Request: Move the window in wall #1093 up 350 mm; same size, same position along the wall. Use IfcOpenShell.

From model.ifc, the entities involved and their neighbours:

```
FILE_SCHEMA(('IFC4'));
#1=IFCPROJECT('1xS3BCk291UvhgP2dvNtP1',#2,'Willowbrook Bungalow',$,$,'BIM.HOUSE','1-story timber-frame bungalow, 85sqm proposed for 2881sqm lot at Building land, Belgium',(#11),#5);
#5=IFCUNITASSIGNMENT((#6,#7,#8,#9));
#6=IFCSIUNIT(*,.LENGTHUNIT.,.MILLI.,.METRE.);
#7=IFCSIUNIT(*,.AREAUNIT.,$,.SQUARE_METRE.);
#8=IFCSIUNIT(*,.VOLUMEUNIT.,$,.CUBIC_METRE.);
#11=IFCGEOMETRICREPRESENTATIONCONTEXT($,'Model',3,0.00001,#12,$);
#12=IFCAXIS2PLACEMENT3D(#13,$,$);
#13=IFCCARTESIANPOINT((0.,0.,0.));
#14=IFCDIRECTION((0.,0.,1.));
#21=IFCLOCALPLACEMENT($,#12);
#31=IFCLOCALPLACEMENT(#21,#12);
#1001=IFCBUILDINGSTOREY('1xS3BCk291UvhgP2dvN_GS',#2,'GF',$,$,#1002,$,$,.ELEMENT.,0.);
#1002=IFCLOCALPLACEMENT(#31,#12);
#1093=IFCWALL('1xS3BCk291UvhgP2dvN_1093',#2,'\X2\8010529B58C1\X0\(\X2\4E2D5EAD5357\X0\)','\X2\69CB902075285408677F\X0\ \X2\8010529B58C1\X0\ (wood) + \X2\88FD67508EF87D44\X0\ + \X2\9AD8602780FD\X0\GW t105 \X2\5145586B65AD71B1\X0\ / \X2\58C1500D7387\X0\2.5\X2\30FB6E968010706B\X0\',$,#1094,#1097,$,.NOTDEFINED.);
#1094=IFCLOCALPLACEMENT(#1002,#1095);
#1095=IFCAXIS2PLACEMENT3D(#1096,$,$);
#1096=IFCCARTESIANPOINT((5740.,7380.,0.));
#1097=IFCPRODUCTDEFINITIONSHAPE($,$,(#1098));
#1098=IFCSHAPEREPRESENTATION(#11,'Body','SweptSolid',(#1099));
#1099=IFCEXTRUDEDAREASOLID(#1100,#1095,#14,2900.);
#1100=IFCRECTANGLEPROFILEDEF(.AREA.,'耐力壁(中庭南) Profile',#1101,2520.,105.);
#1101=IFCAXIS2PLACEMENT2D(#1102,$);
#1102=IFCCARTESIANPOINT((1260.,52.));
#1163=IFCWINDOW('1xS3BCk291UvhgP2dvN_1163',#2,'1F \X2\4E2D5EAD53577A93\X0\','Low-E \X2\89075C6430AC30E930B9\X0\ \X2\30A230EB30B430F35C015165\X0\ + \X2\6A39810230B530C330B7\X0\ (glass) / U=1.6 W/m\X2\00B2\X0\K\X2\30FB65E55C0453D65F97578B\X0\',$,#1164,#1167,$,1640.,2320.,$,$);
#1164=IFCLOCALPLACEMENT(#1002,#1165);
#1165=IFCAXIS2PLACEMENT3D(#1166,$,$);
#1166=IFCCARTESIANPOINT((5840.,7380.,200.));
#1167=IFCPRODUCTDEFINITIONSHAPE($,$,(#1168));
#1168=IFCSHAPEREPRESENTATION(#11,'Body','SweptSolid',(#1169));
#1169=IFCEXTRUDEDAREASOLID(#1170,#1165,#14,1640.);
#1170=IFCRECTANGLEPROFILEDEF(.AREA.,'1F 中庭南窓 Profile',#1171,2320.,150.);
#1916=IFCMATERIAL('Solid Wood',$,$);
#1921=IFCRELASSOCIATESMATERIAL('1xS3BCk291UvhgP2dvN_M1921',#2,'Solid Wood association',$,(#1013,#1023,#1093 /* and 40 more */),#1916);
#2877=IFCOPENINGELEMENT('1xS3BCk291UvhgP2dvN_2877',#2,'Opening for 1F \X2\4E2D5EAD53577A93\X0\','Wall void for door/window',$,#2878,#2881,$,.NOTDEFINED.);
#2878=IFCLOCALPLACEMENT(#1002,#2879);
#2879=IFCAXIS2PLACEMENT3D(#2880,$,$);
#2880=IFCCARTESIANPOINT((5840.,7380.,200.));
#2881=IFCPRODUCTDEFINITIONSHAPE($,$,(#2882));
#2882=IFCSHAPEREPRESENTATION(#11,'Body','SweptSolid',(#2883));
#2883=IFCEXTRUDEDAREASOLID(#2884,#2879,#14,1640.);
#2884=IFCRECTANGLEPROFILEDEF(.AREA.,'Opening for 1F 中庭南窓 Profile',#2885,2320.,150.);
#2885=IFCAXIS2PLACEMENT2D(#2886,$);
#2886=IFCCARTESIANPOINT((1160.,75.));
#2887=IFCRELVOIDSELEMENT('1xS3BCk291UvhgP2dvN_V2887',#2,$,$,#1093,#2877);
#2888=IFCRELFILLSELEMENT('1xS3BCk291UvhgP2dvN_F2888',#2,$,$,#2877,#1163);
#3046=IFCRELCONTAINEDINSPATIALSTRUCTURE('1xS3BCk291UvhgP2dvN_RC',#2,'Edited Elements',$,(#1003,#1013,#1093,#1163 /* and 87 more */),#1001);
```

```python
import numpy as np
import ifcopenshell
import ifcopenshell.api.geometry
import ifcopenshell.util.placement
import ifcopenshell.util.unit

model = ifcopenshell.open("model.ifc")
unit_scale = ifcopenshell.util.unit.calculate_unit_scale(model)

window = model.by_id(1163)
opening = window.FillsVoids[0].RelatingOpeningElement
dz = 350.0

shift = np.array([0.0, 0.0, dz])
# The window is not placed relative to its opening, so move both.
for product in (opening, window):
    matrix = ifcopenshell.util.placement.get_local_placement(product.ObjectPlacement)
    matrix[:3, 3] += shift
    ifcopenshell.api.geometry.edit_object_placement(model, product=product, matrix=matrix, is_si=False)

print(f"moved by {dz * unit_scale:+.3f} m")

model.write("model-out.ifc")
```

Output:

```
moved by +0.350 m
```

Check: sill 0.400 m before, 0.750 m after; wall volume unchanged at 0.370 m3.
